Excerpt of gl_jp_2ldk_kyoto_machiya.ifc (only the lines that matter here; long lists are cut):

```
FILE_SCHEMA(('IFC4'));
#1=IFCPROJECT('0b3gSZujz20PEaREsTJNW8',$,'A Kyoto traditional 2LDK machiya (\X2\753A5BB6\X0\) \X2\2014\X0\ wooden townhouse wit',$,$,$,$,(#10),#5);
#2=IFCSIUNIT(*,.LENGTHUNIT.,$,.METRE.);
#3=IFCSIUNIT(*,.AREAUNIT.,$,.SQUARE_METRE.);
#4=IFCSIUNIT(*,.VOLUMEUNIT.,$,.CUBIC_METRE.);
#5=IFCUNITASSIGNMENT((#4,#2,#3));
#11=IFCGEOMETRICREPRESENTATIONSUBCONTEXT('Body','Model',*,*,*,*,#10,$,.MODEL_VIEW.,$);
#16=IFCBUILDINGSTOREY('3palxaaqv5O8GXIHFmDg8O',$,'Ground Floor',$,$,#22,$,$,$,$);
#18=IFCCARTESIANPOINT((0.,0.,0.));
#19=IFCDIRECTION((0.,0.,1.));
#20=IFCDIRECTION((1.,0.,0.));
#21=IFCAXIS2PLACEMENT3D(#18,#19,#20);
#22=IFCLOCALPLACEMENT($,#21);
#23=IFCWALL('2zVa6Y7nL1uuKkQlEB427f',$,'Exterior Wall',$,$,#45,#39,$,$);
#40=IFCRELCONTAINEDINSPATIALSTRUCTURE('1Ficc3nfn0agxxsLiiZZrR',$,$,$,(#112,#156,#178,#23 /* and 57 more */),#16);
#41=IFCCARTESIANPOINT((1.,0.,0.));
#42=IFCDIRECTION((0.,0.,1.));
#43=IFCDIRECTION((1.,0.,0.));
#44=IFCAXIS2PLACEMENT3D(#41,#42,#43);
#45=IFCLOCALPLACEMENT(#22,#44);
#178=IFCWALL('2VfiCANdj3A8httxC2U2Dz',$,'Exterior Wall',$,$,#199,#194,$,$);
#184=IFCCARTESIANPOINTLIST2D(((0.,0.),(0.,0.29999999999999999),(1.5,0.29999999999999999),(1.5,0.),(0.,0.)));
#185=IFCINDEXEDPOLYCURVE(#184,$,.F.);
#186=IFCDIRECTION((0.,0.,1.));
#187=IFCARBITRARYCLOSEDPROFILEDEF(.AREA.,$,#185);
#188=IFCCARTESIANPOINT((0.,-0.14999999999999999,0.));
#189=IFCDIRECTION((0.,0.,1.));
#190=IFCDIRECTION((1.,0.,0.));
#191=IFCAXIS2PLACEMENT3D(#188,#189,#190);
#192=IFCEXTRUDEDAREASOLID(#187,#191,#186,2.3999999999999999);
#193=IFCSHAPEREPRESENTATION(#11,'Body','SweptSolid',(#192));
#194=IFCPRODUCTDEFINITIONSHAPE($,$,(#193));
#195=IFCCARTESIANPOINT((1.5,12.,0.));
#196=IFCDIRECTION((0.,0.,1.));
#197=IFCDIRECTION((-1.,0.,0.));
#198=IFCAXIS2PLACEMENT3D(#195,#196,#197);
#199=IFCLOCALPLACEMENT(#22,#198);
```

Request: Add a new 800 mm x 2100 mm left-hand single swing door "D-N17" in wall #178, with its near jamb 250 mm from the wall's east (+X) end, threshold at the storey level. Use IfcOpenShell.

```python
import numpy as np
import ifcopenshell
import ifcopenshell.api.feature
import ifcopenshell.api.geometry
import ifcopenshell.api.root
import ifcopenshell.api.spatial
import ifcopenshell.geom
import ifcopenshell.util.element
import ifcopenshell.util.placement
import ifcopenshell.util.representation
import ifcopenshell.util.shape
import ifcopenshell.util.unit

model = ifcopenshell.open("gl_jp_2ldk_kyoto_machiya.ifc")
unit_scale = ifcopenshell.util.unit.calculate_unit_scale(model)
settings = ifcopenshell.geom.settings()


def volume(element):
    """Net volume in cubic metres, openings subtracted."""
    shape = ifcopenshell.geom.create_shape(settings, element)
    return ifcopenshell.util.shape.get_volume(shape.geometry)


wall = model.by_guid("2VfiCANdj3A8httxC2U2Dz")
storey = ifcopenshell.util.element.get_container(wall, ifc_class="IfcBuildingStorey")
context = ifcopenshell.util.representation.get_context(model, "Model", "Body", "MODEL_VIEW")
before = volume(wall)

width, height, from_end, sill = 0.8, 2.1, 0.25, 0.0  # metres

# The wall runs along its own X axis, and the end named is its -X end.
wall_shape = ifcopenshell.geom.create_shape(settings, wall)
x, y, z = ifcopenshell.util.shape.get_vertices(wall_shape.geometry).T
start = x.min() + from_end
face, thickness = float(y.min()), float(y.max() - y.min())
wall_matrix = ifcopenshell.util.placement.get_local_placement(wall.ObjectPlacement)
level = ifcopenshell.util.placement.get_local_placement(storey.ObjectPlacement)[2, 3]


def in_wall(x, y):
    """Placement at x, y metres in the wall's axes, at sill height."""
    matrix = wall_matrix.copy()
    matrix[:, 3] = wall_matrix @ np.array([x / unit_scale, y / unit_scale, 0.0, 1.0])
    matrix[2, 3] = level + sill / unit_scale
    return matrix


# Opening: a box that overshoots both wall faces by 50 mm.
opening = ifcopenshell.api.root.create_entity(model, ifc_class="IfcOpeningElement", predefined_type="OPENING")
box = ifcopenshell.api.geometry.add_wall_representation(
    model, context=context, length=width, height=height, thickness=thickness + 0.1
)
ifcopenshell.api.geometry.assign_representation(model, product=opening, representation=box)
ifcopenshell.api.geometry.edit_object_placement(model, product=opening, matrix=in_wall(start, face - 0.05), is_si=False)
ifcopenshell.api.feature.add_feature(model, feature=opening, element=wall)

door = ifcopenshell.api.root.create_entity(model, ifc_class="IfcDoor", name="D-N17", predefined_type="DOOR")
door.OverallWidth, door.OverallHeight = width / unit_scale, height / unit_scale
door.OperationType = "SINGLE_SWING_LEFT"
body = ifcopenshell.api.geometry.add_door_representation(
    model,
    context=context,
    overall_width=door.OverallWidth,
    overall_height=door.OverallHeight,
    operation_type="SINGLE_SWING_LEFT",
    lining_properties={"LiningDepth": thickness / unit_scale, "ThresholdDepth": thickness / unit_scale},
)
ifcopenshell.api.geometry.assign_representation(model, product=door, representation=body)
ifcopenshell.api.spatial.assign_container(model, products=[door], relating_structure=storey)
ifcopenshell.api.feature.add_filling(model, opening=opening, element=door)

# The lining spans the wall, so the door starts at the wall face.
ifcopenshell.api.geometry.edit_object_placement(model, product=door, matrix=in_wall(start, face), is_si=False)

after = volume(wall)

print(f"wall volume {before:.3f} -> {after:.3f} m3")

model.write("gl_jp_2ldk_kyoto_machiya_edited.ifc")
```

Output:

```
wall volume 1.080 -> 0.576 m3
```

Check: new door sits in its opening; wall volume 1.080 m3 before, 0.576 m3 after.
